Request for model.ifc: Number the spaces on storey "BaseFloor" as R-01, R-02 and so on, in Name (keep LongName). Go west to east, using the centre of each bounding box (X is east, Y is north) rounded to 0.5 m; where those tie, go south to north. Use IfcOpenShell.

First a look at what the model holds.

```python
import ifcopenshell
import ifcopenshell.util.element
import ifcopenshell.util.placement

model = ifcopenshell.open("model.ifc")
print(model.schema)
storey = next(s for s in model.by_type("IfcBuildingStorey") if s.Name == "BaseFloor")
spaces = [e for e in ifcopenshell.util.element.get_decomposition(storey) if e.is_a("IfcSpace")]
for e in sorted(spaces, key=lambda e: e.id()):
    origin = ifcopenshell.util.placement.get_local_placement(e.ObjectPlacement)[:3, 3]
    print(e.id(), e.Name, e.LongName, origin.round(2) + 0.0, sep=" | ")
```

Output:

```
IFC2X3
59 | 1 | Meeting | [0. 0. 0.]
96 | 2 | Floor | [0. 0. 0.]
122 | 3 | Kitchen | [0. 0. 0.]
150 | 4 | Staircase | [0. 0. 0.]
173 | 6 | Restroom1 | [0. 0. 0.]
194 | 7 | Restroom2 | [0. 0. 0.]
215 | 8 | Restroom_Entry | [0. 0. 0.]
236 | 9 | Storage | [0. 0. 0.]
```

```python
import ifcopenshell
import ifcopenshell.geom
import ifcopenshell.util.element
import ifcopenshell.util.shape

model = ifcopenshell.open("model.ifc")
settings = ifcopenshell.geom.settings()
settings.set("use-world-coords", True)


def centre(element):
    shape = ifcopenshell.geom.create_shape(settings, element)
    return ifcopenshell.util.shape.get_bbox_centroid(shape.geometry)


storey = next(s for s in model.by_type("IfcBuildingStorey") if s.Name == "BaseFloor")
spaces = [e for e in ifcopenshell.util.element.get_decomposition(storey) if e.is_a("IfcSpace")]

# Insertion points can sit at a corner or the storey origin, so sort by the geometry (in metres).
centres = {e: centre(e) for e in spaces}
spaces.sort(key=lambda e: (round(centres[e][0] / 0.5), centres[e][1]))

for i, e in enumerate(spaces, start=1):
    number = f"R-{i:02d}"
    e.Name = number
    print(e.id(), number)

model.write("model_rev.ifc")
```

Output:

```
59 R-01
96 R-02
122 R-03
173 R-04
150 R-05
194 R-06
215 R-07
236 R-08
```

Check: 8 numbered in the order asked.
